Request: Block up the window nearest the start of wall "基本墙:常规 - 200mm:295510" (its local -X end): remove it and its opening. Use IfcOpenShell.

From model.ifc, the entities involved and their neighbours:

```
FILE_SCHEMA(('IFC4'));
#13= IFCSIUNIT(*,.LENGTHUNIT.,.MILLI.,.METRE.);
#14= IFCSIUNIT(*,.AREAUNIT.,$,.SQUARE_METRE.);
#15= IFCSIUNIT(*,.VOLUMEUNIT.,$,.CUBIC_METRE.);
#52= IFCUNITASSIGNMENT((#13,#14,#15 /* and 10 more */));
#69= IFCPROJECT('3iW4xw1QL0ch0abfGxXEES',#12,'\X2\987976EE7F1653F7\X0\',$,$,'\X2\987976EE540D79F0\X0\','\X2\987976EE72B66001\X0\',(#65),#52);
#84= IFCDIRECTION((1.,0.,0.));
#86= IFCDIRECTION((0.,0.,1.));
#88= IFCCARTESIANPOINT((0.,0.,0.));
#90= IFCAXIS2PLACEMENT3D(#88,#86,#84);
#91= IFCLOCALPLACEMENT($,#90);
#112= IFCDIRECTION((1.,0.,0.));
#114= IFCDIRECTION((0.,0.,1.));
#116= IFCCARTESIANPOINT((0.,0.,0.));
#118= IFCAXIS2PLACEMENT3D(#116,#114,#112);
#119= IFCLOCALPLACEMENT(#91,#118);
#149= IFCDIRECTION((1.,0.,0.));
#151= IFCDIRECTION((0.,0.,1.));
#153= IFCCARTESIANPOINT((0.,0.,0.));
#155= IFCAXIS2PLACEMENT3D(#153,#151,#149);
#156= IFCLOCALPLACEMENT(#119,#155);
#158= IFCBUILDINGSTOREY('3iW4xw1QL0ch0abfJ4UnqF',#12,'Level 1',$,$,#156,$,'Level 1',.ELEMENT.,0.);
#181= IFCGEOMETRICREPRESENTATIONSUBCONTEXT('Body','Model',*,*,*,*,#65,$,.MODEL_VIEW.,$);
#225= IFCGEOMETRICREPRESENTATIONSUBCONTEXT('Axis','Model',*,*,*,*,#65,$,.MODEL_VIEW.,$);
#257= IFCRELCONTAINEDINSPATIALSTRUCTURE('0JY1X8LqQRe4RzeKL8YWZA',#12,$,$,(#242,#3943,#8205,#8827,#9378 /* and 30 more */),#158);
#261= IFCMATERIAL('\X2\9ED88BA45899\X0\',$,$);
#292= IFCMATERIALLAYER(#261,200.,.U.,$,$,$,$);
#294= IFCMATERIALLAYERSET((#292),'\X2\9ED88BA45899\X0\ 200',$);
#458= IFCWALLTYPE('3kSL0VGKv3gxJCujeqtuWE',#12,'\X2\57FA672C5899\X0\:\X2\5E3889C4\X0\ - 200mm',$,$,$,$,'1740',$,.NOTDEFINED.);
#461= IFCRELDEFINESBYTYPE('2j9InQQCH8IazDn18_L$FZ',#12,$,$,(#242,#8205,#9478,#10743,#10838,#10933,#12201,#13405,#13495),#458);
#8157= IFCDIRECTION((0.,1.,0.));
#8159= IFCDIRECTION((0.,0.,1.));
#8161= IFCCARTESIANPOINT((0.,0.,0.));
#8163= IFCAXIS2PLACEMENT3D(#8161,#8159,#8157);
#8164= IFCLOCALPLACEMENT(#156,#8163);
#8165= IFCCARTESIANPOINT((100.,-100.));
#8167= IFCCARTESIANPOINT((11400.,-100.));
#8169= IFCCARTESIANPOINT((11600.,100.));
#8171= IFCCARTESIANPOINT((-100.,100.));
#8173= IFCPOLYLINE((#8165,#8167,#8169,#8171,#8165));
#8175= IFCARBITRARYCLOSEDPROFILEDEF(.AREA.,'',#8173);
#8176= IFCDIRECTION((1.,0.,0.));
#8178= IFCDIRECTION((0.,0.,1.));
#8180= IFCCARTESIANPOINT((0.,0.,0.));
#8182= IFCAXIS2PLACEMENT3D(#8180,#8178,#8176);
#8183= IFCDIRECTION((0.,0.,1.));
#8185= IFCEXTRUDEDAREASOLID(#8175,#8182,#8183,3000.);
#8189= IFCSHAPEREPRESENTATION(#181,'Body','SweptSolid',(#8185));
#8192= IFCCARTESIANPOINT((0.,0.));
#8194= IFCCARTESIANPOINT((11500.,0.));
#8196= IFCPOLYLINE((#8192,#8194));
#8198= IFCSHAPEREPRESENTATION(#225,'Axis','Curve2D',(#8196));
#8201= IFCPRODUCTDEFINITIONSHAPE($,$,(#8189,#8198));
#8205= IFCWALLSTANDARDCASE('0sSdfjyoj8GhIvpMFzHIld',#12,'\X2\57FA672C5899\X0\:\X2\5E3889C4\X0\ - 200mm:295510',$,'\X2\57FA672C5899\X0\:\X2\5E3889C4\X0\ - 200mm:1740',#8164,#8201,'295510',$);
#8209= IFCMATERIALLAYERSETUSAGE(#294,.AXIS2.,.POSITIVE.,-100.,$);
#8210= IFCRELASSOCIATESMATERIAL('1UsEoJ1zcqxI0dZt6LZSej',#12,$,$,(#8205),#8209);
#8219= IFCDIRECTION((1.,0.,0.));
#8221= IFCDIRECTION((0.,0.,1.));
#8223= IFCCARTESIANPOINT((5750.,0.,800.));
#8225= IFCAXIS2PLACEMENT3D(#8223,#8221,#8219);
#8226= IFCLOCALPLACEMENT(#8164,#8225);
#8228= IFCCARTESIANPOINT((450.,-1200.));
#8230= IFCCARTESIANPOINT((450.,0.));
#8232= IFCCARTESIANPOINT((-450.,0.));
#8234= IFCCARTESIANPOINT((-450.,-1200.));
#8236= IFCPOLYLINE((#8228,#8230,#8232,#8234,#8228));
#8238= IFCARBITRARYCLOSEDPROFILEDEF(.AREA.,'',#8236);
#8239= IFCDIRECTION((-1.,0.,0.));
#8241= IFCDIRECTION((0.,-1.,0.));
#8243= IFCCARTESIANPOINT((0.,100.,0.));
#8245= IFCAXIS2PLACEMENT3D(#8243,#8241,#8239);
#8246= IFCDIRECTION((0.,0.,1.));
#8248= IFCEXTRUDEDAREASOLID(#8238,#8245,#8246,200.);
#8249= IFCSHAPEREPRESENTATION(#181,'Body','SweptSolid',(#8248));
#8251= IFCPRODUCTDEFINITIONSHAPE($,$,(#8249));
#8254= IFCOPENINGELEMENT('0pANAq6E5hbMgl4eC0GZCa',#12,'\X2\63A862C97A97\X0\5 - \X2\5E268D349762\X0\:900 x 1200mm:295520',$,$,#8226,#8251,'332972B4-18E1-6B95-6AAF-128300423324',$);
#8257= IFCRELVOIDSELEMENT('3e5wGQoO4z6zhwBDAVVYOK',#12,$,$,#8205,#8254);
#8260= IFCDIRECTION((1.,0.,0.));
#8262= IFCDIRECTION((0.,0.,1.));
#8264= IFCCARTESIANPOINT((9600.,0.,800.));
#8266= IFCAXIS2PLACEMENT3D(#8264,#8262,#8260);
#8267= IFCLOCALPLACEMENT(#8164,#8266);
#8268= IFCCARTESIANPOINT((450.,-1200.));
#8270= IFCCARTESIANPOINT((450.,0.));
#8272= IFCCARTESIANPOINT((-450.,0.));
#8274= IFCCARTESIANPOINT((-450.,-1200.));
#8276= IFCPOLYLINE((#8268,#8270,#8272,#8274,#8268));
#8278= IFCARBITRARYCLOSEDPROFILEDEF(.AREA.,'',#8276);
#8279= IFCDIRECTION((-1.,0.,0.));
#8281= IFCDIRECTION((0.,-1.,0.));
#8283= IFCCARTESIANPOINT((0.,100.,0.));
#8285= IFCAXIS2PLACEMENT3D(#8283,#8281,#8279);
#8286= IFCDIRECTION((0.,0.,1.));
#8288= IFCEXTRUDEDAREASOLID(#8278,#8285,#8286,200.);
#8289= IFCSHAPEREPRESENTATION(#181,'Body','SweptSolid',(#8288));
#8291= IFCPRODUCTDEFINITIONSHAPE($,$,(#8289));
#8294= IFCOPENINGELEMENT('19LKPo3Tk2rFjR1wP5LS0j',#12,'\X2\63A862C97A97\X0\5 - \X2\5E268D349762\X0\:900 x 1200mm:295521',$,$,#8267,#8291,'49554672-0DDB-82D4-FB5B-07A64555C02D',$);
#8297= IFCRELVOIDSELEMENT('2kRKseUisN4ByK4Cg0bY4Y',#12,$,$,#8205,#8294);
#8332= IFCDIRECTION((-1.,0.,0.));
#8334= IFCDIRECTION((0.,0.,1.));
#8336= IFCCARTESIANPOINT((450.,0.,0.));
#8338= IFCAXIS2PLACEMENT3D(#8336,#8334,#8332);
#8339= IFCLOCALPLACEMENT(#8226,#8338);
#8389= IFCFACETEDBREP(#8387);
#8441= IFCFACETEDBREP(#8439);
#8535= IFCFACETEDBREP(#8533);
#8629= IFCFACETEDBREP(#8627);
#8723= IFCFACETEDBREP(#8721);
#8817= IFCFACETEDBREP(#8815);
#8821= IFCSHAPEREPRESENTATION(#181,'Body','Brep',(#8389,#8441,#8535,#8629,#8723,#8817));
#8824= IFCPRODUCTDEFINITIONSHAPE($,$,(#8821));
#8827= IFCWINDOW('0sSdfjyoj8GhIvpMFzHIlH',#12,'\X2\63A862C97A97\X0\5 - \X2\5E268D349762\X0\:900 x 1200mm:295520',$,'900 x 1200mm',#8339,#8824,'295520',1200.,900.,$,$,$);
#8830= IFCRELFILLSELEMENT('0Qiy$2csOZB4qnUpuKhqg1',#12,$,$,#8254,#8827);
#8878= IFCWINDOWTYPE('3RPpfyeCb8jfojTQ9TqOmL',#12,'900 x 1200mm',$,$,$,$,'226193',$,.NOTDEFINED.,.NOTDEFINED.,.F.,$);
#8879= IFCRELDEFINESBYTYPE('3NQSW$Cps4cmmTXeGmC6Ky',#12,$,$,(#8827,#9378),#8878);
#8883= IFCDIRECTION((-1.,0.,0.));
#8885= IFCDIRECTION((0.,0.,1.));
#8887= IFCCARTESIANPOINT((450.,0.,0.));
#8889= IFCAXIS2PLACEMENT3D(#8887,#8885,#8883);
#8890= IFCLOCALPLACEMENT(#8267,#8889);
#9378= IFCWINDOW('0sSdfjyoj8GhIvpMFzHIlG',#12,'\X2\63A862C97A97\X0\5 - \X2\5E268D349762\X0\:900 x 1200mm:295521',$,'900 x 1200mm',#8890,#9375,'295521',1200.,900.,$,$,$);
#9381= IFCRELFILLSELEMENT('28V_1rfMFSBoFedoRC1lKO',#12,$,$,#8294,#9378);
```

```python
import ifcopenshell
import ifcopenshell.api.feature
import ifcopenshell.api.root
import ifcopenshell.geom
import ifcopenshell.util.shape

model = ifcopenshell.open("model.ifc")
settings = ifcopenshell.geom.settings()


def volume(element):
    """Net volume in cubic metres, openings subtracted."""
    shape = ifcopenshell.geom.create_shape(settings, element)
    return ifcopenshell.util.shape.get_volume(shape.geometry)


window = model.by_guid("0sSdfjyoj8GhIvpMFzHIlH")
opening = window.FillsVoids[0].RelatingOpeningElement
wall = opening.VoidsElements[0].RelatingBuildingElement
before = volume(wall)

ifcopenshell.api.root.remove_product(model, product=window)
ifcopenshell.api.feature.remove_feature(model, feature=opening)

after = volume(wall)

print(f"wall volume {before:.3f} -> {after:.3f} m3")

model.write("model-out.ifc")
```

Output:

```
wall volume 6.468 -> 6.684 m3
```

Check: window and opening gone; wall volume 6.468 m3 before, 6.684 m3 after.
